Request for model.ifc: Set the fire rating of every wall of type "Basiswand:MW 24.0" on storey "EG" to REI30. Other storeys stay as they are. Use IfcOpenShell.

First a look at what the model holds.

```python
import ifcopenshell
import ifcopenshell.util.element

model = ifcopenshell.open("model.ifc")
print(model.schema)
storey = next(s for s in model.by_type("IfcBuildingStorey") if s.Name == "EG")
walls = [e for e in ifcopenshell.util.element.get_decomposition(storey) if e.is_a("IfcWall")]
seen = {}
for e in walls:
    element_type = ifcopenshell.util.element.get_type(e)
    key = (element_type.Name if element_type != e and element_type else None, ifcopenshell.util.element.get_pset(e, "Pset_WallCommon", "FireRating"))
    seen[key] = seen.get(key, 0) + 1
for (name, value), count in sorted(seen.items(), key=str):
    print(count, "x", name, "|", value)
```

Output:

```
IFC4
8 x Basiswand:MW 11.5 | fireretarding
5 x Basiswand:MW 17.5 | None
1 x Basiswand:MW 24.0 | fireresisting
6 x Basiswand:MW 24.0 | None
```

```python
import ifcopenshell
import ifcopenshell.api.pset
import ifcopenshell.util.element

model = ifcopenshell.open("model.ifc")

storey = next(s for s in model.by_type("IfcBuildingStorey") if s.Name == "EG")
walls = [e for e in ifcopenshell.util.element.get_decomposition(storey) if e.is_a("IfcWall")]

count = 0
for e in walls:
    element_type = ifcopenshell.util.element.get_type(e)
    if element_type in (None, e) or element_type.Name != "Basiswand:MW 24.0":
        continue
    # add_pset returns the element's existing set when there is one.
    pset = ifcopenshell.api.pset.add_pset(model, product=e, name="Pset_WallCommon")
    ifcopenshell.api.pset.edit_pset(model, pset=pset, properties={"FireRating": "REI30"})
    count += 1

print(count, "walls updated")

model.write("model-out.ifc")
```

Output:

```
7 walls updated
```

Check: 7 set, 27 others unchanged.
